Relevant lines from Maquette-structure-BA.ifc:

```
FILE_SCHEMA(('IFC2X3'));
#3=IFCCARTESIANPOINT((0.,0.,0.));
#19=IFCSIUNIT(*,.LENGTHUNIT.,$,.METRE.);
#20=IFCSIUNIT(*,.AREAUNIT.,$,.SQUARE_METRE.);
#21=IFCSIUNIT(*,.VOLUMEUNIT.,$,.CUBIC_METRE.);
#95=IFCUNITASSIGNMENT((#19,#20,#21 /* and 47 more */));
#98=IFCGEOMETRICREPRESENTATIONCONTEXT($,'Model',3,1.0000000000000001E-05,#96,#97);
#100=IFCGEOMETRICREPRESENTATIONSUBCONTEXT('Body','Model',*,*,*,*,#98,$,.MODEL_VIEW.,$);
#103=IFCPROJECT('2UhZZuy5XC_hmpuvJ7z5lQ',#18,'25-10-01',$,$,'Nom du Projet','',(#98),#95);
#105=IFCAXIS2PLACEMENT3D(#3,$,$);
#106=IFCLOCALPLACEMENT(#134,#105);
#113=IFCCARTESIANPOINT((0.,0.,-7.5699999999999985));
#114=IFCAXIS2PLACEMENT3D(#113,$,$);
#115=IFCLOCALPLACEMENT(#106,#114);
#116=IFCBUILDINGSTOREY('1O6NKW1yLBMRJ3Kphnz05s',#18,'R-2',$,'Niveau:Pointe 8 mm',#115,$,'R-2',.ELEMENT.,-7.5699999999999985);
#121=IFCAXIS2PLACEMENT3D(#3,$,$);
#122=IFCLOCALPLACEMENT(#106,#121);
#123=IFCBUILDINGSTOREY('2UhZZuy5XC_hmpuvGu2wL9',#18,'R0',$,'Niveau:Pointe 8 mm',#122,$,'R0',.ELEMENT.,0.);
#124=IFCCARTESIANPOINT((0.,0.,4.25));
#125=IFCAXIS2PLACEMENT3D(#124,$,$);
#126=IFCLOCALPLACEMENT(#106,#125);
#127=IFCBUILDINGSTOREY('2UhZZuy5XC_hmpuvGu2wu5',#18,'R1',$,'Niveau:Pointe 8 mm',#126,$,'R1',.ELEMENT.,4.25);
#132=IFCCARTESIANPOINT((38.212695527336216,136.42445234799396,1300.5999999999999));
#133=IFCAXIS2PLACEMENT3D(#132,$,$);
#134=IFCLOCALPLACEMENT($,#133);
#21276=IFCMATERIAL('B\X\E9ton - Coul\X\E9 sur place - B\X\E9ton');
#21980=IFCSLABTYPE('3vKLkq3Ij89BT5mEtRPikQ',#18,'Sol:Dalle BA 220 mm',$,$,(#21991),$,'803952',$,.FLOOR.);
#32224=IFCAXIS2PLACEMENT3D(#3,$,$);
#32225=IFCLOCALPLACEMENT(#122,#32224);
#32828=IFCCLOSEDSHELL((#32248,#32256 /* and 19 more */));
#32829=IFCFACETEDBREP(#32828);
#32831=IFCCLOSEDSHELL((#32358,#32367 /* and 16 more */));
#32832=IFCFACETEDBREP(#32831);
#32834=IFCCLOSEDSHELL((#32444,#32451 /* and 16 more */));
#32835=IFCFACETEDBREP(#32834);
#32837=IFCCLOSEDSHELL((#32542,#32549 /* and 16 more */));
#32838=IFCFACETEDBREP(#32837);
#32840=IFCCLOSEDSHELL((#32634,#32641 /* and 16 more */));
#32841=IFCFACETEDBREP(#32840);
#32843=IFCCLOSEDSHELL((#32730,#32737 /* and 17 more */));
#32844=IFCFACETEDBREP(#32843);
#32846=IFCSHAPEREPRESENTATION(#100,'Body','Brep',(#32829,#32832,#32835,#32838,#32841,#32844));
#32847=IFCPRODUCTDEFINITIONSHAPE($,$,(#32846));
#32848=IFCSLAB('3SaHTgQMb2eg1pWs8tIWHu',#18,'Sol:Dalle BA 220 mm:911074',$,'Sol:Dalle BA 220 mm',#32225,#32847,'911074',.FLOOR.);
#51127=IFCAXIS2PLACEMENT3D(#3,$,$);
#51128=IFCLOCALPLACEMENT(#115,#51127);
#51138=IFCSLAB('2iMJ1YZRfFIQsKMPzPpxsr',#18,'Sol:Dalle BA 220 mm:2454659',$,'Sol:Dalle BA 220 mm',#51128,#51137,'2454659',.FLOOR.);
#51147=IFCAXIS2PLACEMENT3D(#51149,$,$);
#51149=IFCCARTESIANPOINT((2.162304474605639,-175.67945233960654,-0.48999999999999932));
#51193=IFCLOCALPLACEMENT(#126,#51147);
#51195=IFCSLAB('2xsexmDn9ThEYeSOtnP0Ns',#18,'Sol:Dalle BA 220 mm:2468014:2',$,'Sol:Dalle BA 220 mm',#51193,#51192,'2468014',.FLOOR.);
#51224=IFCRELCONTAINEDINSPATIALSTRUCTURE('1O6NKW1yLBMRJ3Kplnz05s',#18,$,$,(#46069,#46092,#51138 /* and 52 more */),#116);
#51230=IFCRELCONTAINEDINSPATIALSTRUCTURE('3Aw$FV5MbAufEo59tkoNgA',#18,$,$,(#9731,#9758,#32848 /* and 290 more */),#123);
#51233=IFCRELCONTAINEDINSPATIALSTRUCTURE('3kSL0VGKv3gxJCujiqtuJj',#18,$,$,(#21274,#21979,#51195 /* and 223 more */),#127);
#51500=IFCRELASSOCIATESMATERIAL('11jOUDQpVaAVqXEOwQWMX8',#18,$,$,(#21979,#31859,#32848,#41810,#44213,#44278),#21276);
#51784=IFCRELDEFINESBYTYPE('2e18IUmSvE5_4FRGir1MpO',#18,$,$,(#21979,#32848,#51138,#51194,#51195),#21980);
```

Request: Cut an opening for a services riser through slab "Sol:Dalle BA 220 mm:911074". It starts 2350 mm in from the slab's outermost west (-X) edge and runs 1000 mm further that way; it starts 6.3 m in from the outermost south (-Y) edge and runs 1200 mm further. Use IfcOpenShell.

```python
import numpy as np
import ifcopenshell
import ifcopenshell.api.feature
import ifcopenshell.api.geometry
import ifcopenshell.api.root
import ifcopenshell.geom
import ifcopenshell.util.placement
import ifcopenshell.util.representation
import ifcopenshell.util.shape
import ifcopenshell.util.unit

model = ifcopenshell.open("Maquette-structure-BA.ifc")
unit_scale = ifcopenshell.util.unit.calculate_unit_scale(model)
settings = ifcopenshell.geom.settings()


def volume(element):
    """Net volume in cubic metres, openings subtracted."""
    shape = ifcopenshell.geom.create_shape(settings, element)
    return ifcopenshell.util.shape.get_volume(shape.geometry)


slab = model.by_guid("3SaHTgQMb2eg1pWs8tIWHu")
before = volume(slab)

# Extent in the slab's own axes, in metres. The edges named are its -X and -Y sides.
slab_shape = ifcopenshell.geom.create_shape(settings, slab)
vertices = ifcopenshell.util.shape.get_vertices(slab_shape.geometry)
x_min, y_min, bottom = vertices.min(axis=0)
top = vertices[:, 2].max()

opening = ifcopenshell.api.root.create_entity(model, ifc_class="IfcOpeningElement", name="Services riser opening")
context = ifcopenshell.util.representation.get_context(model, "Model", "Body", "MODEL_VIEW")
width, depth = 1, 1.2
outline = [(0.0, 0.0), (width, 0.0), (width, depth), (0.0, depth), (0.0, 0.0)]
# Overshoot both faces by 50 mm so the cut is clean.
shape = ifcopenshell.api.geometry.add_slab_representation(
    model, context=context, depth=top - bottom + 0.1, polyline=outline
)
ifcopenshell.api.geometry.assign_representation(model, product=opening, representation=shape)

matrix = ifcopenshell.util.placement.get_local_placement(slab.ObjectPlacement)
matrix[:, 3] = matrix @ np.append(np.array([x_min + 2.35, y_min + 6.3, bottom - 0.05]) / unit_scale, 1.0)
ifcopenshell.api.geometry.edit_object_placement(model, product=opening, matrix=matrix, is_si=False)
ifcopenshell.api.feature.add_feature(model, feature=opening, element=slab)

after = volume(slab)

print(f"slab volume {before:.3f} -> {after:.3f} m3")

model.write("Maquette-structure-BA_rev.ifc")
```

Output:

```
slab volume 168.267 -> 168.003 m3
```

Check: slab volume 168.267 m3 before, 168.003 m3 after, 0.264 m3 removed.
